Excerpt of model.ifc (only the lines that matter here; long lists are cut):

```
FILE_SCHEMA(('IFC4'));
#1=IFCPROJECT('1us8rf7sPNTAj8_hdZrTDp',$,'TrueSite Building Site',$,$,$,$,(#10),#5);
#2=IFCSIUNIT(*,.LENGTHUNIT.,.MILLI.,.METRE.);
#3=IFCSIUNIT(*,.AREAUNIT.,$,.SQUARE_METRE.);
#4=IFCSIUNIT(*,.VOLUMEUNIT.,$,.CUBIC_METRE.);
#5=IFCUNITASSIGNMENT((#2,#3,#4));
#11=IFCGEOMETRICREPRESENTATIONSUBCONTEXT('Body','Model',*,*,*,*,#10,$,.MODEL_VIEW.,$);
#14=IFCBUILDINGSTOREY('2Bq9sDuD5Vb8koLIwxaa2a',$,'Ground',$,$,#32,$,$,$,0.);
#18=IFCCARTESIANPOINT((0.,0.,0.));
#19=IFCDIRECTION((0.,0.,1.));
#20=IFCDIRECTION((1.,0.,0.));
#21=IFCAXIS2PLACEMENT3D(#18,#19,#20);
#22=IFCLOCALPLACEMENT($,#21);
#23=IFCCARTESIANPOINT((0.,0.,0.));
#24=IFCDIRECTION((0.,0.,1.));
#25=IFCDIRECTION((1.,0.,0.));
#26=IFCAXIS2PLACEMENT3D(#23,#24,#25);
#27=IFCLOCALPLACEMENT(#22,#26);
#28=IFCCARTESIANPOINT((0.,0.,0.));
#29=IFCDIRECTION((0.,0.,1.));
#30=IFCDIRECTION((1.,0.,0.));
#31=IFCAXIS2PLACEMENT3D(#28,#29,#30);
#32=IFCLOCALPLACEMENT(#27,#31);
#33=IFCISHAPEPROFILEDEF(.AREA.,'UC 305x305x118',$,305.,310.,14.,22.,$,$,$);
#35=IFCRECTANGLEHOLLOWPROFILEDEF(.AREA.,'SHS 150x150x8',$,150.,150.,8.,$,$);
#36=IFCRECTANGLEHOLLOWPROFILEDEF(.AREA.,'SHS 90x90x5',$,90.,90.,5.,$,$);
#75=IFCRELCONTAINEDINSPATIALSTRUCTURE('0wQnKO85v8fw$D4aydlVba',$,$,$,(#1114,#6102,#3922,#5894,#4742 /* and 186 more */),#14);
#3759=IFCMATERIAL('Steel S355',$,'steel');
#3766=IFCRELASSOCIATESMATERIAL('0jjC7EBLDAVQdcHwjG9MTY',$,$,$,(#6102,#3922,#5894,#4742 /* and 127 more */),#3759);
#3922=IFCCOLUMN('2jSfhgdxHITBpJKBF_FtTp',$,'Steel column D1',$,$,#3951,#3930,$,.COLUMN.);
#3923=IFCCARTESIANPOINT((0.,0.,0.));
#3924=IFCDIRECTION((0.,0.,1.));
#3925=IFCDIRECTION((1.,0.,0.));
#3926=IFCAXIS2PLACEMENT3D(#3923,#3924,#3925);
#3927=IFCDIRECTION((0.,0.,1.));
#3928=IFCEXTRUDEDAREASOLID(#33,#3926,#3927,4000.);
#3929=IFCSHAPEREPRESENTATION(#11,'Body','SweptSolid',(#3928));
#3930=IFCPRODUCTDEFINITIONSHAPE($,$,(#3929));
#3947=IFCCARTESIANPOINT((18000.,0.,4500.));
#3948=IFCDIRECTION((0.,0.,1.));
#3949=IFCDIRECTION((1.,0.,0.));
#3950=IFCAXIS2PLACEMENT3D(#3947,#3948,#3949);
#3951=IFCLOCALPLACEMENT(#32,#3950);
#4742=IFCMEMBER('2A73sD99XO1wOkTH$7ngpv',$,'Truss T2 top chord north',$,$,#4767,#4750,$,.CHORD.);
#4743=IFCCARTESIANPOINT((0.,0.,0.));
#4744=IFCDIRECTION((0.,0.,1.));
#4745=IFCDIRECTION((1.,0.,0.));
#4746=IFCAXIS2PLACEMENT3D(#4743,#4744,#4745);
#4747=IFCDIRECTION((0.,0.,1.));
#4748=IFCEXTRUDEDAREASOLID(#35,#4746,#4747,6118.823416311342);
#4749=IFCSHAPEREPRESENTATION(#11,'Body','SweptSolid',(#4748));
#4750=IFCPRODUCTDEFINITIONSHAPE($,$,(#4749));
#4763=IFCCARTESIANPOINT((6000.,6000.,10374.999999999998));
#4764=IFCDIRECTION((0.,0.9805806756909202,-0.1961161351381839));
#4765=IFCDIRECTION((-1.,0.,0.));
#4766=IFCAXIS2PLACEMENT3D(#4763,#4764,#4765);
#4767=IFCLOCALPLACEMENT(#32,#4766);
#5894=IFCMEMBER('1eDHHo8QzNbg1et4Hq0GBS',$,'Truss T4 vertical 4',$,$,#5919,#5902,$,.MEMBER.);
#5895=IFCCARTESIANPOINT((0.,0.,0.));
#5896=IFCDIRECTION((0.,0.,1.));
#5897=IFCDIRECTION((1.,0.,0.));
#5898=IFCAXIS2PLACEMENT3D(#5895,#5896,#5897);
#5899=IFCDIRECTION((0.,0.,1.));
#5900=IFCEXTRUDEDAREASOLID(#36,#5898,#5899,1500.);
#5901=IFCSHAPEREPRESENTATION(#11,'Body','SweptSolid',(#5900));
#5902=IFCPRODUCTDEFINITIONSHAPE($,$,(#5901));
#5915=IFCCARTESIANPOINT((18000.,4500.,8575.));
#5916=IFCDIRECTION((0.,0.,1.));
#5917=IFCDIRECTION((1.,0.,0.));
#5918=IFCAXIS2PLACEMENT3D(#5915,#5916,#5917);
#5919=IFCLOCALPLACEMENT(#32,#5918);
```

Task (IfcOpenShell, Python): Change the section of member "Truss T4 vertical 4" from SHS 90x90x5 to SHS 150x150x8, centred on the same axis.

```python
import ifcopenshell
import ifcopenshell.util.element
import ifcopenshell.util.representation

model = ifcopenshell.open("model.ifc")

member = model.by_guid("1eDHHo8QzNbg1et4Hq0GBS")
source = next(p for p in model.by_type("IfcRectangleHollowProfileDef") if p.ProfileName == "SHS 150x150x8")

body = ifcopenshell.util.representation.get_representation(member, "Model", "Body")
solid = body.Items[0]
old_profile = solid.SweptArea

# Copy the section's sizes but keep this member's own profile position.
profile = ifcopenshell.util.element.copy(model, source)
profile.Position = old_profile.Position
solid.SweptArea = profile
if not model.get_total_inverses(old_profile):
    ifcopenshell.util.element.remove_deep2(model, old_profile)

print(solid.SweptArea)

model.write("model_v2.ifc")
```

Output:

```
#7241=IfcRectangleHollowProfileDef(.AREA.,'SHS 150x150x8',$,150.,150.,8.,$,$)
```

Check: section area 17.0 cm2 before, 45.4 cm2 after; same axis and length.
